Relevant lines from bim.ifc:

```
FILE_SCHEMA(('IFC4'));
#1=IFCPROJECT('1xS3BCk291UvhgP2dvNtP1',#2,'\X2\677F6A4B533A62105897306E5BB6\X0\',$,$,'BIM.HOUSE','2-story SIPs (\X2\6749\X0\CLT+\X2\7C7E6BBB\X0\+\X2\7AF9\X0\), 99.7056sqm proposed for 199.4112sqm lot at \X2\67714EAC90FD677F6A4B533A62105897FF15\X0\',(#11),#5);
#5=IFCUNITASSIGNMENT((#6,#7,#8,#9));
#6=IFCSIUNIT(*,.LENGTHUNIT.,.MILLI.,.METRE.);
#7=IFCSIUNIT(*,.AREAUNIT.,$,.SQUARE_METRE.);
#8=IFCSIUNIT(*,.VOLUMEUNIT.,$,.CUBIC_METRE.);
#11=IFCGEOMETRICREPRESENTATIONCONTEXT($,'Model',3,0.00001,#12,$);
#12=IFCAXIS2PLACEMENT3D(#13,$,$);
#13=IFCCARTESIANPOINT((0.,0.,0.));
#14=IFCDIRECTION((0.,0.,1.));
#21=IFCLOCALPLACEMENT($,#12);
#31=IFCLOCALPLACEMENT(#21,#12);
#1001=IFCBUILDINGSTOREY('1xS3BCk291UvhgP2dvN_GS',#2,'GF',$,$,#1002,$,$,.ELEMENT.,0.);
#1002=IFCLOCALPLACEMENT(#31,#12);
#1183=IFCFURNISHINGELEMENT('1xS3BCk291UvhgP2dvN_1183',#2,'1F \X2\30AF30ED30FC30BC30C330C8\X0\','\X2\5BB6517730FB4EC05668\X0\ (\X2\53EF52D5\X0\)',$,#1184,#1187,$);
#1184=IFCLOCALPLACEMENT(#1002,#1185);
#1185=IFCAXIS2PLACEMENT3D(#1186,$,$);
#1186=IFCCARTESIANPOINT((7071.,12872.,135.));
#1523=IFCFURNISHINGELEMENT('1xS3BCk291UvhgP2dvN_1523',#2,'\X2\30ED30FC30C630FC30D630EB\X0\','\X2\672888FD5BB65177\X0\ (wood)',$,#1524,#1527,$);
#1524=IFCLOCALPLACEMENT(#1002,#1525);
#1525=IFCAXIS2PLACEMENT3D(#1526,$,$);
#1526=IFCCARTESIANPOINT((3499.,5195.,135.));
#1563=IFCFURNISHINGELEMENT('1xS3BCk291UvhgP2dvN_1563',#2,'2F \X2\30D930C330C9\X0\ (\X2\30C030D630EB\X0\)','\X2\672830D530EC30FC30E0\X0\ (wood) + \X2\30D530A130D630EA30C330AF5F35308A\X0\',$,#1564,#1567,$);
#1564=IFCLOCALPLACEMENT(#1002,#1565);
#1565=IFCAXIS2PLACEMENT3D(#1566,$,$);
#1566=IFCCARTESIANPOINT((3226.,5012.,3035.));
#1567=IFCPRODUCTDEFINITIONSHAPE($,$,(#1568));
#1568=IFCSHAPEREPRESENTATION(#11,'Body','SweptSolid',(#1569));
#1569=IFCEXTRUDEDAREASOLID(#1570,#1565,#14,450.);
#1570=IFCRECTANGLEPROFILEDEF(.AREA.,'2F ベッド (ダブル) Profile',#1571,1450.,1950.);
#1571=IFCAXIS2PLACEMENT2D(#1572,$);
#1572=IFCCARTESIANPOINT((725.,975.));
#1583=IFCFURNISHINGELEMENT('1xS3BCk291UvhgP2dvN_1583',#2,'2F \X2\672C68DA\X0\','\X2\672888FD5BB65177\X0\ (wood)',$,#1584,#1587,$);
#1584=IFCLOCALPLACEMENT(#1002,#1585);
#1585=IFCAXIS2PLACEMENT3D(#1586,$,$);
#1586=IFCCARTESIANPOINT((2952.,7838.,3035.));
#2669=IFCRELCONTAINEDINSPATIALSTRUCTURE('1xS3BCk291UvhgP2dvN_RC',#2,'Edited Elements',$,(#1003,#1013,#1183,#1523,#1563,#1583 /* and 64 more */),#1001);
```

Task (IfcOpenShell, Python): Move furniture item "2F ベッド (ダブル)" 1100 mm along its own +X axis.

```python
import ifcopenshell
import ifcopenshell.api.geometry
import ifcopenshell.util.placement

model = ifcopenshell.open("bim.ifc")

item = model.by_id(1563)
matrix = ifcopenshell.util.placement.get_local_placement(item.ObjectPlacement)
matrix[:3, 3] += matrix[:3, 0] * 1100.0
ifcopenshell.api.geometry.edit_object_placement(model, product=item, matrix=matrix, is_si=False)

print(ifcopenshell.util.placement.get_local_placement(item.ObjectPlacement).round(3) + 0.0)

model.write("bim_rev.ifc")
```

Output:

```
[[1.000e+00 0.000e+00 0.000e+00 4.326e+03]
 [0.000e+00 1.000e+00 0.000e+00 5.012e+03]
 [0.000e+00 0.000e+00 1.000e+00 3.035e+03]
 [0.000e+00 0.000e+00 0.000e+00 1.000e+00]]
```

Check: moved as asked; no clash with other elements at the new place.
